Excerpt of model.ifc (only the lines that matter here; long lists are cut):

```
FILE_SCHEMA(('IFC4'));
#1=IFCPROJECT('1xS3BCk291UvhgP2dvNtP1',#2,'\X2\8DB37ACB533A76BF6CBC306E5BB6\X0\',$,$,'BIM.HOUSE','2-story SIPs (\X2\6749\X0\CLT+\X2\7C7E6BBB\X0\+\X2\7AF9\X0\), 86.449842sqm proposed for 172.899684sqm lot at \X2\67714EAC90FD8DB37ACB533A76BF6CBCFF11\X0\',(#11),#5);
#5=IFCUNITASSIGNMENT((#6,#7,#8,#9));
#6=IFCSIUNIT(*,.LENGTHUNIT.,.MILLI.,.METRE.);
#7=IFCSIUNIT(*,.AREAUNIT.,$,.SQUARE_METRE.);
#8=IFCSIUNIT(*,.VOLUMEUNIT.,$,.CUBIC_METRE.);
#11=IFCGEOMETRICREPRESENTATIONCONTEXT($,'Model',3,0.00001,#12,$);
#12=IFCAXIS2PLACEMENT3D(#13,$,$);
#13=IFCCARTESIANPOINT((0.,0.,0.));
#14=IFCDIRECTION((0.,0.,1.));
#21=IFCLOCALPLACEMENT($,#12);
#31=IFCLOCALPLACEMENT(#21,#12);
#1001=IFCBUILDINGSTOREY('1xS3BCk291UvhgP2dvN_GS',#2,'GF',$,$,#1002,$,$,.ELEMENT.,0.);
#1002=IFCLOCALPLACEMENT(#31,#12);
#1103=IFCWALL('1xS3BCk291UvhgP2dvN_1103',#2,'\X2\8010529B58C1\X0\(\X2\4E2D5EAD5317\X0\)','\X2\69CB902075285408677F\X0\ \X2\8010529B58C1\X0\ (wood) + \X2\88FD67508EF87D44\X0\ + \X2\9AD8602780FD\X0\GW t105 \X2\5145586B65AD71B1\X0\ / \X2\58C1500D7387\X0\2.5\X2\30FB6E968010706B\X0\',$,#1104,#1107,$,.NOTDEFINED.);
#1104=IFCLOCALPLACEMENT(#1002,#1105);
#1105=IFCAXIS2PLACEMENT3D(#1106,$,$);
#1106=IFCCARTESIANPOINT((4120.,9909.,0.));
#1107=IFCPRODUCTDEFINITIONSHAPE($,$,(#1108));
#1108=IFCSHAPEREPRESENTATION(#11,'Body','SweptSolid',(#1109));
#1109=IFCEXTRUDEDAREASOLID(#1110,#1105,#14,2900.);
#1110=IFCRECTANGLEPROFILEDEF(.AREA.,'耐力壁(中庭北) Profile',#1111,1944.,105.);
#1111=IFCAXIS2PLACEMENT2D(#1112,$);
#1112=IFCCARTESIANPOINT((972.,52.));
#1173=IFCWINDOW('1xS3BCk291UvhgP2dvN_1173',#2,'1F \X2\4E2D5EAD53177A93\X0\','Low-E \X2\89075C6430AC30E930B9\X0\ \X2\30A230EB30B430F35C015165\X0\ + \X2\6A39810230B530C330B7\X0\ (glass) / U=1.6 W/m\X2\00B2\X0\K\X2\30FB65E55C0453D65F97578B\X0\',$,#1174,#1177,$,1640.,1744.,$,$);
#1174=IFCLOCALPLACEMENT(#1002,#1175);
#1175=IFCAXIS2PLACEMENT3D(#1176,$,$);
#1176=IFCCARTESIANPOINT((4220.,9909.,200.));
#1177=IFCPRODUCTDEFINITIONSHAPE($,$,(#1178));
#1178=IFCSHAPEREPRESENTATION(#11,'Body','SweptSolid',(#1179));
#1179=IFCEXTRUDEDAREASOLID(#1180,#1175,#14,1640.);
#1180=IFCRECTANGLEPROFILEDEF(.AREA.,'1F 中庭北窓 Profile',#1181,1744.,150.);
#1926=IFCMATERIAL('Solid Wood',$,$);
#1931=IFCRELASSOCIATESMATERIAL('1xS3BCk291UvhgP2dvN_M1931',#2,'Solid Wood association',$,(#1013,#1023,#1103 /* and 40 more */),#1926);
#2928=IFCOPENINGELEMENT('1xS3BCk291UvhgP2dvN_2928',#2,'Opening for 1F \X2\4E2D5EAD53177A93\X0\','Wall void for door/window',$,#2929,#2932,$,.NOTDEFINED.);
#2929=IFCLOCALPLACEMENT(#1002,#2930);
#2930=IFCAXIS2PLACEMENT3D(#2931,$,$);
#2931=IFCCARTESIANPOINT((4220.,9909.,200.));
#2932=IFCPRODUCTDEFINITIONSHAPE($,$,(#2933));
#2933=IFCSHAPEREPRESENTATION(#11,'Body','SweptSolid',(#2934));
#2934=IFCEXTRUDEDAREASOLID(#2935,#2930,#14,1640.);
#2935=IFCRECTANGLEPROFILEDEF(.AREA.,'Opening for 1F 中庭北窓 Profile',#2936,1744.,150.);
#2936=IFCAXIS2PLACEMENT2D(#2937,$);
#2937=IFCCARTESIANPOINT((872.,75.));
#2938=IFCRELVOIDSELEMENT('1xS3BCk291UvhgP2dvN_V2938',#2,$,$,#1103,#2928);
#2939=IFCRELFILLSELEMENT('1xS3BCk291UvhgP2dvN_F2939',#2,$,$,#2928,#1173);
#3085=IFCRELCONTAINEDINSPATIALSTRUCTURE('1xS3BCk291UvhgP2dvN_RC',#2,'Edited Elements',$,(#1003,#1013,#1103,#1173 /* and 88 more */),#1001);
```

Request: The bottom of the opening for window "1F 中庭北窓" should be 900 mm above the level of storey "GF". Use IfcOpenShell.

```python
import numpy as np
import ifcopenshell
import ifcopenshell.api.geometry
import ifcopenshell.geom
import ifcopenshell.util.element
import ifcopenshell.util.placement
import ifcopenshell.util.shape
import ifcopenshell.util.unit

model = ifcopenshell.open("model.ifc")
unit_scale = ifcopenshell.util.unit.calculate_unit_scale(model)

window = model.by_guid("1xS3BCk291UvhgP2dvN_1173")
opening = window.FillsVoids[0].RelatingOpeningElement
storey = ifcopenshell.util.element.get_container(window, ifc_class="IfcBuildingStorey")
level = ifcopenshell.util.placement.get_local_placement(storey.ObjectPlacement)[2, 3]

# The opening's origin need not be at the sill, so measure its lowest point.
shape = ifcopenshell.geom.create_shape(ifcopenshell.geom.settings(), opening)
bottom = ifcopenshell.util.shape.get_shape_bottom_elevation(shape, shape.geometry) / unit_scale
dz = level + 0.9 / unit_scale - bottom

shift = np.array([0.0, 0.0, dz])
# The window is not placed relative to its opening, so move both.
for product in (opening, window):
    matrix = ifcopenshell.util.placement.get_local_placement(product.ObjectPlacement)
    matrix[:3, 3] += shift
    ifcopenshell.api.geometry.edit_object_placement(model, product=product, matrix=matrix, is_si=False)

print(f"moved by {dz * unit_scale:+.3f} m")

model.write("model_rev.ifc")
```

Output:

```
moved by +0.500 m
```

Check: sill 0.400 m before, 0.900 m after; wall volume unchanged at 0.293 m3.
